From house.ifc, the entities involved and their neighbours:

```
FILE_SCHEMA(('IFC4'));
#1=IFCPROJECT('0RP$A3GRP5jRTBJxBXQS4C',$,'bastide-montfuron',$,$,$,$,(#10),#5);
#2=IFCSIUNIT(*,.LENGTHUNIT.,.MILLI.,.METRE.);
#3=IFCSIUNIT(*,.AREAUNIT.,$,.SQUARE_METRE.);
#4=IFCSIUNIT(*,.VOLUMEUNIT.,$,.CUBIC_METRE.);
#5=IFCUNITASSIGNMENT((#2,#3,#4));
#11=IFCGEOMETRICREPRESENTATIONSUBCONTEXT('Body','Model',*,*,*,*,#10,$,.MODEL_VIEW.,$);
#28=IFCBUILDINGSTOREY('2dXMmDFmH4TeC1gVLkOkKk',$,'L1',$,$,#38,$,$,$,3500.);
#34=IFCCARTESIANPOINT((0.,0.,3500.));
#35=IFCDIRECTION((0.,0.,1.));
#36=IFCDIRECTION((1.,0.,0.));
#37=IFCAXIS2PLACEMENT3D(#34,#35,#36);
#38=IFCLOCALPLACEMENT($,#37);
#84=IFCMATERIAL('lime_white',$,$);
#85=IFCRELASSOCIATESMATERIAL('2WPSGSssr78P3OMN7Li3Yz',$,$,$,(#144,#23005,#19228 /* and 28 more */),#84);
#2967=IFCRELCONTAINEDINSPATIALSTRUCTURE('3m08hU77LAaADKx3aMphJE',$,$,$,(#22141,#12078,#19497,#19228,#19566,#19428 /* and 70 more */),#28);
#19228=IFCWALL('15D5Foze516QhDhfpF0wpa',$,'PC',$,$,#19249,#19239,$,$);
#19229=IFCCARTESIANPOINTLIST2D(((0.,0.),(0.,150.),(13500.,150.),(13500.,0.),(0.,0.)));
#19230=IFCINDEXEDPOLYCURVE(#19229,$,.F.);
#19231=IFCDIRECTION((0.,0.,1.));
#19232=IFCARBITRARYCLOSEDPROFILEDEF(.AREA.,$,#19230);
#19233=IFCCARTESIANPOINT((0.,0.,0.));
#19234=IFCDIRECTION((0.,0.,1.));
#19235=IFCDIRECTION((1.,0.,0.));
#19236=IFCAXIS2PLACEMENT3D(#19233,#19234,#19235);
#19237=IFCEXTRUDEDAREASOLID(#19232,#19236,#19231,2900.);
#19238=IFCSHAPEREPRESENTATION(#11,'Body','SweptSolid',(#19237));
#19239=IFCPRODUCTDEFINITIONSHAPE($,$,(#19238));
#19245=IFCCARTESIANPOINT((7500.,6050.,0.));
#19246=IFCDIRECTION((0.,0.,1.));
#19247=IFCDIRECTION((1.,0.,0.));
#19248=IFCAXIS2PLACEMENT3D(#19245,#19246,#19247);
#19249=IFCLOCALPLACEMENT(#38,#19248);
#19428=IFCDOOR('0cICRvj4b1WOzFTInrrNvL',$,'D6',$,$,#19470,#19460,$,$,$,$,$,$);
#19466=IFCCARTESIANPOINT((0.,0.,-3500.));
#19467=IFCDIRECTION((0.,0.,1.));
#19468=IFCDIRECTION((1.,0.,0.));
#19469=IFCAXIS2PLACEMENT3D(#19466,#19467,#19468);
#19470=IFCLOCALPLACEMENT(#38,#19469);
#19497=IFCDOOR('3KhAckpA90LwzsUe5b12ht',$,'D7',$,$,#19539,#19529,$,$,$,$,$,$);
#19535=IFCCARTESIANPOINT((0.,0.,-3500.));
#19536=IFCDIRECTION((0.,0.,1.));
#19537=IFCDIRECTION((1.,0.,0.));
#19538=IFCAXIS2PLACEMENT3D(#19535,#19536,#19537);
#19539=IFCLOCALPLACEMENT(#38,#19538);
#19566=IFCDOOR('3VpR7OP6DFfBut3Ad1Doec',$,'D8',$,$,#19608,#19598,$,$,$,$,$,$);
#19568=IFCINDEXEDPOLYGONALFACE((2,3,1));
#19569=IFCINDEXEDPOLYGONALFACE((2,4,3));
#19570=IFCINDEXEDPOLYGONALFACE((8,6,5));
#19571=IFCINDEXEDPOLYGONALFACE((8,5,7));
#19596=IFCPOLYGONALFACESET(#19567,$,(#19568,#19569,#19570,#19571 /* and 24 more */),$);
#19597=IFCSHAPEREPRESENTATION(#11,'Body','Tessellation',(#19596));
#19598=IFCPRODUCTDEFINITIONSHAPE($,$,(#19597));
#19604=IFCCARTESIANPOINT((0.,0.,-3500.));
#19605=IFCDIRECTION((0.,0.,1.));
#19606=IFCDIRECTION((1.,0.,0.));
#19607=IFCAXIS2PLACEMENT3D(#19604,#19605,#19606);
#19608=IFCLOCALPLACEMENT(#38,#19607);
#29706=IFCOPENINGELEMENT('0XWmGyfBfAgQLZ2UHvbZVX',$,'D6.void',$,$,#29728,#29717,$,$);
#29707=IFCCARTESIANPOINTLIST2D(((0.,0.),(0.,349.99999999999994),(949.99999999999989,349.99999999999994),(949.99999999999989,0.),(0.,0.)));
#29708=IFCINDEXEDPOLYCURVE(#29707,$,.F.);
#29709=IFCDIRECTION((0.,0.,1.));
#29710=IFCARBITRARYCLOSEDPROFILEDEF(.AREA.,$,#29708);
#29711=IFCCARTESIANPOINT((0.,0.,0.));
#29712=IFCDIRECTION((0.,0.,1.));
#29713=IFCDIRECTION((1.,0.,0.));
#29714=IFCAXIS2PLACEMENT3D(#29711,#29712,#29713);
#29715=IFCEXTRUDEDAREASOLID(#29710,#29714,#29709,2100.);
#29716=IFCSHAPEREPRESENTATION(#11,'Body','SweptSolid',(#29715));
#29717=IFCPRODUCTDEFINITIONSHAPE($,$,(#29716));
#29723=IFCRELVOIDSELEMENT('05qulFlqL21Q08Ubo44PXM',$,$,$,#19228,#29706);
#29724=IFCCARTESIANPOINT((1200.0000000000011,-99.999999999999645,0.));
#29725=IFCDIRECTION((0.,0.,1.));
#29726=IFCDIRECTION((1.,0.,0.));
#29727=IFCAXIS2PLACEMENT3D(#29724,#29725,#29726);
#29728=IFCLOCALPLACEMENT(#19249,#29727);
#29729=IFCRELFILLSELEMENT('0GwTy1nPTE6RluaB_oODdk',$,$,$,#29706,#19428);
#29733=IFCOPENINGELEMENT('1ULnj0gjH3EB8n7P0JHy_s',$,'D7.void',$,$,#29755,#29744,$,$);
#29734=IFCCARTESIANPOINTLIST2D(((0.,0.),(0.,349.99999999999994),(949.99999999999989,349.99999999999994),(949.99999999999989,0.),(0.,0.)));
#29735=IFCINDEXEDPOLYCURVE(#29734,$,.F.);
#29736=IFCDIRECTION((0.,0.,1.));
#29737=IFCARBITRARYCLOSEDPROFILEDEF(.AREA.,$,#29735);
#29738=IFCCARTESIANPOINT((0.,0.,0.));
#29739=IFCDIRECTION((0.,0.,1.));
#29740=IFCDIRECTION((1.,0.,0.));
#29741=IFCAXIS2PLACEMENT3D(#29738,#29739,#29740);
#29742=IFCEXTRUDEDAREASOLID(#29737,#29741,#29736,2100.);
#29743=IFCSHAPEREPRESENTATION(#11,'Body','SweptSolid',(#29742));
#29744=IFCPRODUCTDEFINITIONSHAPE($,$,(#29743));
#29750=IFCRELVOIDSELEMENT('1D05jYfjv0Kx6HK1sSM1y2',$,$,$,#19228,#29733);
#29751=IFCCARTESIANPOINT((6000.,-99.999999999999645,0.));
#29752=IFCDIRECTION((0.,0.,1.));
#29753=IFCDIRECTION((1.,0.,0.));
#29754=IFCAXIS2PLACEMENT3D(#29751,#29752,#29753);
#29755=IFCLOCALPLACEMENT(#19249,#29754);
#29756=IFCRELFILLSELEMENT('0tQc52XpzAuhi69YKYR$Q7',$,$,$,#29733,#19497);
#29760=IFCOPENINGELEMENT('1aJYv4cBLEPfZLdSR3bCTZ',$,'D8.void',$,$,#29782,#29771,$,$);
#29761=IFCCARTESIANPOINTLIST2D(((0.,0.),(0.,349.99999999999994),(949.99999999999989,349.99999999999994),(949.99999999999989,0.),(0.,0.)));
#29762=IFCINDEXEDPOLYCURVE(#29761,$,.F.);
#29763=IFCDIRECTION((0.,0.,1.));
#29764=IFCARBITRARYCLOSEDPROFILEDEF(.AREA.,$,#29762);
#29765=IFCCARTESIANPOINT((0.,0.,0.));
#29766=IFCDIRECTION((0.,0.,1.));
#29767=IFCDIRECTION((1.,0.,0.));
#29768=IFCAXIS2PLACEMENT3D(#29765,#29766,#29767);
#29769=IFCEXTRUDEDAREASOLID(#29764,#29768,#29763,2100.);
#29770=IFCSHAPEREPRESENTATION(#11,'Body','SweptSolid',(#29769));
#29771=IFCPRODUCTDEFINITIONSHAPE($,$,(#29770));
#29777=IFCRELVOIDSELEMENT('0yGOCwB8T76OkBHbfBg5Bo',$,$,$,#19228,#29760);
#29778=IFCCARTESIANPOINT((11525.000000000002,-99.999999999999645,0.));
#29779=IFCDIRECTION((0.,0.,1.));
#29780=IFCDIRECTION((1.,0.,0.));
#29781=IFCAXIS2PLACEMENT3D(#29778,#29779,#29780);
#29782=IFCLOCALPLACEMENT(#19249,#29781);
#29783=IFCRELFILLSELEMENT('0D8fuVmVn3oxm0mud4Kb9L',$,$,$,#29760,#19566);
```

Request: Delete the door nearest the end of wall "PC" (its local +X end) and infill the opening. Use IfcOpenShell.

```python
import ifcopenshell
import ifcopenshell.api.feature
import ifcopenshell.api.root
import ifcopenshell.geom
import ifcopenshell.util.shape

model = ifcopenshell.open("house.ifc")
settings = ifcopenshell.geom.settings()


def volume(element):
    """Net volume in cubic metres, openings subtracted."""
    shape = ifcopenshell.geom.create_shape(settings, element)
    return ifcopenshell.util.shape.get_volume(shape.geometry)


door = model.by_id(19566)
opening = door.FillsVoids[0].RelatingOpeningElement
wall = opening.VoidsElements[0].RelatingBuildingElement
before = volume(wall)

ifcopenshell.api.root.remove_product(model, product=door)
ifcopenshell.api.feature.remove_feature(model, feature=opening)

after = volume(wall)

print(f"wall volume {before:.3f} -> {after:.3f} m3")

model.write("house_edited.ifc")
```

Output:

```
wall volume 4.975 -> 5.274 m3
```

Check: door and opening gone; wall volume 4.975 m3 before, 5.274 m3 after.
